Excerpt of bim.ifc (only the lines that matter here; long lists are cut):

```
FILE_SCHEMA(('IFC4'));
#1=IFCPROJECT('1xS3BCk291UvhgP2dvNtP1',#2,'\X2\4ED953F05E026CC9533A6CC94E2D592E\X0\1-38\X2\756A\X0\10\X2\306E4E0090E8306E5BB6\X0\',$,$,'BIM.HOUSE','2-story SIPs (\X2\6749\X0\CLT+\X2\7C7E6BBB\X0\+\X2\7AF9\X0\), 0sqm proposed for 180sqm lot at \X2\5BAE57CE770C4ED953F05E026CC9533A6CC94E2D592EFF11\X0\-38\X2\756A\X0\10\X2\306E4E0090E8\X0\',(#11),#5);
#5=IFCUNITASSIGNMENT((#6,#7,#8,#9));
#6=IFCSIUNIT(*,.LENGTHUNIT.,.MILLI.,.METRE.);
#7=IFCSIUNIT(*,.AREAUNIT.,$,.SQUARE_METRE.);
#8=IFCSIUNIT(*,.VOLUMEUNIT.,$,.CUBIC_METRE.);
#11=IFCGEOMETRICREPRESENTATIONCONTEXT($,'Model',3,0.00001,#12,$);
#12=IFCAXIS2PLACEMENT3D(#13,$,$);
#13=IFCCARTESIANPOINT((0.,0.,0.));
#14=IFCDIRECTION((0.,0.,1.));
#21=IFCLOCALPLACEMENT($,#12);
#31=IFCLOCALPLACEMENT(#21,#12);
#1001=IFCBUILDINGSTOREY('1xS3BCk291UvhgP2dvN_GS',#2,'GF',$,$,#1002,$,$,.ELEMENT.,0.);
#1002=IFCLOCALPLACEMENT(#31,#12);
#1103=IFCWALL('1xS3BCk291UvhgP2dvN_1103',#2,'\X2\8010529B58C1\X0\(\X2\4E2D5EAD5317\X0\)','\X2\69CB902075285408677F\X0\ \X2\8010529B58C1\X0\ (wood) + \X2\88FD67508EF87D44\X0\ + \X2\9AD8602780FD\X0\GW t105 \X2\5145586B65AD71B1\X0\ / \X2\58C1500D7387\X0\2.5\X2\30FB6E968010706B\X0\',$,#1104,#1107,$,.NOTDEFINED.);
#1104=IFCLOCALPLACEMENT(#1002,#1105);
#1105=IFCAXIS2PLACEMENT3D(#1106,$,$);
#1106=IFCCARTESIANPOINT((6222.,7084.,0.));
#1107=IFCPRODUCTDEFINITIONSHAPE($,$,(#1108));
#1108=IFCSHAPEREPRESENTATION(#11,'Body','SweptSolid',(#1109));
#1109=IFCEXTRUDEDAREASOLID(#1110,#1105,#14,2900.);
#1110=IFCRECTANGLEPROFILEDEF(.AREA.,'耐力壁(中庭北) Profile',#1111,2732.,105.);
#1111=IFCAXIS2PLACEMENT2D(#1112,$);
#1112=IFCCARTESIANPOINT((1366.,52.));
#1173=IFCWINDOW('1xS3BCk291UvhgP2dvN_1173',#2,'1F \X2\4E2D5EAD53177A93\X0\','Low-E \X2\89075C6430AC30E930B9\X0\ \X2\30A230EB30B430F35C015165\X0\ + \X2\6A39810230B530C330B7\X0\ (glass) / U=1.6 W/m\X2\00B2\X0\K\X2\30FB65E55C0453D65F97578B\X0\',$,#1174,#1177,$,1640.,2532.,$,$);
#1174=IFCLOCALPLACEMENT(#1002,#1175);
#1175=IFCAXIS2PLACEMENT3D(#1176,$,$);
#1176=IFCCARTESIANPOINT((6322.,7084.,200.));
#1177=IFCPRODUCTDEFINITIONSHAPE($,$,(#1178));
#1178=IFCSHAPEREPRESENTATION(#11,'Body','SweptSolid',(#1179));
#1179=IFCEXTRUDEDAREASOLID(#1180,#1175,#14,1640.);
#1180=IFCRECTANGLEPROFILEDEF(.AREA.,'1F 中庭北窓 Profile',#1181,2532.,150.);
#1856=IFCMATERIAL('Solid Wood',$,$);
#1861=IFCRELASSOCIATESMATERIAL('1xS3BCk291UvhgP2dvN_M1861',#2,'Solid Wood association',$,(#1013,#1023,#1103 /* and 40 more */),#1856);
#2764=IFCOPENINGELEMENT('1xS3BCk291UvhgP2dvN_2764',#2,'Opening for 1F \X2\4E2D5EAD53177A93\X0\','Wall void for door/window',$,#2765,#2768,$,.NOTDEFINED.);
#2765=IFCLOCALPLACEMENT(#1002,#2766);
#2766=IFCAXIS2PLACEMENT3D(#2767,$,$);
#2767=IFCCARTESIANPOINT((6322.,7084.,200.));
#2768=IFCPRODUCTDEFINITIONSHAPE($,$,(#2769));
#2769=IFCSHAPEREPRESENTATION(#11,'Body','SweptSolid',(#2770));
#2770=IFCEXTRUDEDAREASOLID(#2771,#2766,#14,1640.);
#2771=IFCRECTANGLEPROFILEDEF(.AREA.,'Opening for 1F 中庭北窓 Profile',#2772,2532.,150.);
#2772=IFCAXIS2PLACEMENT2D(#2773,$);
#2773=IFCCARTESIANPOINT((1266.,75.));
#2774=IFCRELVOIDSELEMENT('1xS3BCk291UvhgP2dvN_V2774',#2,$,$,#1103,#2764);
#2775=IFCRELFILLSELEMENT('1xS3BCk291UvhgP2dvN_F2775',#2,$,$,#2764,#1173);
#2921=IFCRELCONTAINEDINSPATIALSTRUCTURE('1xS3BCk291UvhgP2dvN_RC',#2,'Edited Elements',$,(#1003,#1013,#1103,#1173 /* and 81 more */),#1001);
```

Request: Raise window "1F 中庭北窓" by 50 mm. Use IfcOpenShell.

```python
import numpy as np
import ifcopenshell
import ifcopenshell.api.geometry
import ifcopenshell.util.placement
import ifcopenshell.util.unit

model = ifcopenshell.open("bim.ifc")
unit_scale = ifcopenshell.util.unit.calculate_unit_scale(model)

window = model.by_id(1173)
opening = window.FillsVoids[0].RelatingOpeningElement
dz = 50.0

shift = np.array([0.0, 0.0, dz])
# The window is not placed relative to its opening, so move both.
for product in (opening, window):
    matrix = ifcopenshell.util.placement.get_local_placement(product.ObjectPlacement)
    matrix[:3, 3] += shift
    ifcopenshell.api.geometry.edit_object_placement(model, product=product, matrix=matrix, is_si=False)

print(f"moved by {dz * unit_scale:+.3f} m")

model.write("bim-out.ifc")
```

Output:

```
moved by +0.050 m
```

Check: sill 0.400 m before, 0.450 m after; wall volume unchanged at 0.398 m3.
